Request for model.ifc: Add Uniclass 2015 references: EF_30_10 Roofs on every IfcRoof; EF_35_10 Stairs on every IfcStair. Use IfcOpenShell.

First a look at what the model holds.

```python
import ifcopenshell

model = ifcopenshell.open("model.ifc")
print(model.schema)
print("classifications:", [c.Name for c in model.by_type("IfcClassification")])
for ifc_class in ("IfcDoor", "IfcRoof", "IfcStair", "IfcWall", "IfcWindow"):
    print(ifc_class, len(model.by_type(ifc_class)))
```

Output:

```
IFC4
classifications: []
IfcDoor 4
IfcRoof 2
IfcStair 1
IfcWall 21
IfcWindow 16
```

```python
import ifcopenshell
import ifcopenshell.api.classification

model = ifcopenshell.open("model.ifc")

system = ifcopenshell.api.classification.add_classification(model, classification="Uniclass 2015")

codes = {
    "IfcRoof": ("EF_30_10", "Roofs"),
    "IfcStair": ("EF_35_10", "Stairs"),
}
for ifc_class, (code, name) in codes.items():
    products = model.by_type(ifc_class)
    ifcopenshell.api.classification.add_reference(
        model, products=products, classification=system, identification=code, name=name
    )
    print(code, len(products))

model.write("model_v2.ifc")
```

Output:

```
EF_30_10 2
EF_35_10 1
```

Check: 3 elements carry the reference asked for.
